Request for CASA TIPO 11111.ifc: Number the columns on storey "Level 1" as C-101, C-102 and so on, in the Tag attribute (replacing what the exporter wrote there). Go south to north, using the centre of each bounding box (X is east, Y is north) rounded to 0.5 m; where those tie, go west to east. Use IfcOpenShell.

First a look at what the model holds.

```python
import ifcopenshell
import ifcopenshell.util.element
import ifcopenshell.util.placement

model = ifcopenshell.open("CASA TIPO 11111.ifc")
print(model.schema)
storey = next(s for s in model.by_type("IfcBuildingStorey") if s.Name == "Level 1")
columns = [e for e in ifcopenshell.util.element.get_decomposition(storey) if e.is_a("IfcColumn")]
for e in sorted(columns, key=lambda e: e.id()):
    origin = ifcopenshell.util.placement.get_local_placement(e.ObjectPlacement)[:3, 3]
    print(e.id(), e.Tag, e.Name, origin.round(2) + 0.0, sep=" | ")
```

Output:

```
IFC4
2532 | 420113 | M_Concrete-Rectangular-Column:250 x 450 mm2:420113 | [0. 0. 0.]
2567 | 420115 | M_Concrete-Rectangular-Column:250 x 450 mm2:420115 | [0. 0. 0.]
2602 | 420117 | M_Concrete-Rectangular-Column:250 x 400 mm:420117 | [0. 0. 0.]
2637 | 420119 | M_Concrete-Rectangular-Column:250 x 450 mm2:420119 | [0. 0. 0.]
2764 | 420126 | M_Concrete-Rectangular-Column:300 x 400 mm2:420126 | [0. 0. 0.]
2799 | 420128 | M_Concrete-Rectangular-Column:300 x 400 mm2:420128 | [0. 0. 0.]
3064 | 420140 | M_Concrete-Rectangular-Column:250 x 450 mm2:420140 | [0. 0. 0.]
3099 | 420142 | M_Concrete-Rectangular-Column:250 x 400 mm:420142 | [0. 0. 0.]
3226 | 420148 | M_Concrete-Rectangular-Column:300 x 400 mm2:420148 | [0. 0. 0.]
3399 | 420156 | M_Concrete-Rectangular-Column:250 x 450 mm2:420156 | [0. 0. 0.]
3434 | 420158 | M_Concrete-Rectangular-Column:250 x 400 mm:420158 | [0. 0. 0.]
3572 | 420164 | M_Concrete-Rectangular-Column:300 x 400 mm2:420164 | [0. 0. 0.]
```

```python
import ifcopenshell
import ifcopenshell.geom
import ifcopenshell.util.element
import ifcopenshell.util.shape

model = ifcopenshell.open("CASA TIPO 11111.ifc")
settings = ifcopenshell.geom.settings()
settings.set("use-world-coords", True)


def centre(element):
    shape = ifcopenshell.geom.create_shape(settings, element)
    return ifcopenshell.util.shape.get_bbox_centroid(shape.geometry)


storey = next(s for s in model.by_type("IfcBuildingStorey") if s.Name == "Level 1")
columns = [e for e in ifcopenshell.util.element.get_decomposition(storey) if e.is_a("IfcColumn")]

# Insertion points can sit at a corner or the storey origin, so sort by the geometry (in metres).
centres = {e: centre(e) for e in columns}
columns.sort(key=lambda e: (round(centres[e][1] / 0.5), centres[e][0]))

for i, e in enumerate(columns, start=1):
    number = f"C-1{i:02d}"
    e.Tag = number
    print(e.id(), number)

model.write("CASA TIPO 11111_updated.ifc")
```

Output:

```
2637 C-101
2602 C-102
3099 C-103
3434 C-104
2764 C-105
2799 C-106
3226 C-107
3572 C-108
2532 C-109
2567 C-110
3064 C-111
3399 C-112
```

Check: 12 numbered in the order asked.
